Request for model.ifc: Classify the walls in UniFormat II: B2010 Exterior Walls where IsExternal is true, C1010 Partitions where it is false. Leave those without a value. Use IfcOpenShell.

First a look at what the model holds.

```python
import ifcopenshell
import ifcopenshell.util.element

model = ifcopenshell.open("model.ifc")
print(model.schema)
print("classifications:", [c.Name for c in model.by_type("IfcClassification")])
values = [ifcopenshell.util.element.get_pset(e, "Pset_WallCommon", "IsExternal") for e in model.by_type("IfcWall")]
for value in (True, False, None):
    print("IsExternal", value, values.count(value))
```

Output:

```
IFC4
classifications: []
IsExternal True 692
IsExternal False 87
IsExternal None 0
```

```python
import ifcopenshell
import ifcopenshell.api.classification
import ifcopenshell.util.element

model = ifcopenshell.open("model.ifc")

system = ifcopenshell.api.classification.add_classification(model, classification="UniFormat II")

walls = model.by_type("IfcWall")
external = {e: ifcopenshell.util.element.get_pset(e, "Pset_WallCommon", "IsExternal") for e in walls}
for flag, code, name in ((True, "B2010", "Exterior Walls"), (False, "C1010", "Partitions")):
    products = [e for e in walls if external[e] is flag]
    ifcopenshell.api.classification.add_reference(
        model, products=products, classification=system, identification=code, name=name
    )
    print(code, len(products))

model.write("model_rev.ifc")
```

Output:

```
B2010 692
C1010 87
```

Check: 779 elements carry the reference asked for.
